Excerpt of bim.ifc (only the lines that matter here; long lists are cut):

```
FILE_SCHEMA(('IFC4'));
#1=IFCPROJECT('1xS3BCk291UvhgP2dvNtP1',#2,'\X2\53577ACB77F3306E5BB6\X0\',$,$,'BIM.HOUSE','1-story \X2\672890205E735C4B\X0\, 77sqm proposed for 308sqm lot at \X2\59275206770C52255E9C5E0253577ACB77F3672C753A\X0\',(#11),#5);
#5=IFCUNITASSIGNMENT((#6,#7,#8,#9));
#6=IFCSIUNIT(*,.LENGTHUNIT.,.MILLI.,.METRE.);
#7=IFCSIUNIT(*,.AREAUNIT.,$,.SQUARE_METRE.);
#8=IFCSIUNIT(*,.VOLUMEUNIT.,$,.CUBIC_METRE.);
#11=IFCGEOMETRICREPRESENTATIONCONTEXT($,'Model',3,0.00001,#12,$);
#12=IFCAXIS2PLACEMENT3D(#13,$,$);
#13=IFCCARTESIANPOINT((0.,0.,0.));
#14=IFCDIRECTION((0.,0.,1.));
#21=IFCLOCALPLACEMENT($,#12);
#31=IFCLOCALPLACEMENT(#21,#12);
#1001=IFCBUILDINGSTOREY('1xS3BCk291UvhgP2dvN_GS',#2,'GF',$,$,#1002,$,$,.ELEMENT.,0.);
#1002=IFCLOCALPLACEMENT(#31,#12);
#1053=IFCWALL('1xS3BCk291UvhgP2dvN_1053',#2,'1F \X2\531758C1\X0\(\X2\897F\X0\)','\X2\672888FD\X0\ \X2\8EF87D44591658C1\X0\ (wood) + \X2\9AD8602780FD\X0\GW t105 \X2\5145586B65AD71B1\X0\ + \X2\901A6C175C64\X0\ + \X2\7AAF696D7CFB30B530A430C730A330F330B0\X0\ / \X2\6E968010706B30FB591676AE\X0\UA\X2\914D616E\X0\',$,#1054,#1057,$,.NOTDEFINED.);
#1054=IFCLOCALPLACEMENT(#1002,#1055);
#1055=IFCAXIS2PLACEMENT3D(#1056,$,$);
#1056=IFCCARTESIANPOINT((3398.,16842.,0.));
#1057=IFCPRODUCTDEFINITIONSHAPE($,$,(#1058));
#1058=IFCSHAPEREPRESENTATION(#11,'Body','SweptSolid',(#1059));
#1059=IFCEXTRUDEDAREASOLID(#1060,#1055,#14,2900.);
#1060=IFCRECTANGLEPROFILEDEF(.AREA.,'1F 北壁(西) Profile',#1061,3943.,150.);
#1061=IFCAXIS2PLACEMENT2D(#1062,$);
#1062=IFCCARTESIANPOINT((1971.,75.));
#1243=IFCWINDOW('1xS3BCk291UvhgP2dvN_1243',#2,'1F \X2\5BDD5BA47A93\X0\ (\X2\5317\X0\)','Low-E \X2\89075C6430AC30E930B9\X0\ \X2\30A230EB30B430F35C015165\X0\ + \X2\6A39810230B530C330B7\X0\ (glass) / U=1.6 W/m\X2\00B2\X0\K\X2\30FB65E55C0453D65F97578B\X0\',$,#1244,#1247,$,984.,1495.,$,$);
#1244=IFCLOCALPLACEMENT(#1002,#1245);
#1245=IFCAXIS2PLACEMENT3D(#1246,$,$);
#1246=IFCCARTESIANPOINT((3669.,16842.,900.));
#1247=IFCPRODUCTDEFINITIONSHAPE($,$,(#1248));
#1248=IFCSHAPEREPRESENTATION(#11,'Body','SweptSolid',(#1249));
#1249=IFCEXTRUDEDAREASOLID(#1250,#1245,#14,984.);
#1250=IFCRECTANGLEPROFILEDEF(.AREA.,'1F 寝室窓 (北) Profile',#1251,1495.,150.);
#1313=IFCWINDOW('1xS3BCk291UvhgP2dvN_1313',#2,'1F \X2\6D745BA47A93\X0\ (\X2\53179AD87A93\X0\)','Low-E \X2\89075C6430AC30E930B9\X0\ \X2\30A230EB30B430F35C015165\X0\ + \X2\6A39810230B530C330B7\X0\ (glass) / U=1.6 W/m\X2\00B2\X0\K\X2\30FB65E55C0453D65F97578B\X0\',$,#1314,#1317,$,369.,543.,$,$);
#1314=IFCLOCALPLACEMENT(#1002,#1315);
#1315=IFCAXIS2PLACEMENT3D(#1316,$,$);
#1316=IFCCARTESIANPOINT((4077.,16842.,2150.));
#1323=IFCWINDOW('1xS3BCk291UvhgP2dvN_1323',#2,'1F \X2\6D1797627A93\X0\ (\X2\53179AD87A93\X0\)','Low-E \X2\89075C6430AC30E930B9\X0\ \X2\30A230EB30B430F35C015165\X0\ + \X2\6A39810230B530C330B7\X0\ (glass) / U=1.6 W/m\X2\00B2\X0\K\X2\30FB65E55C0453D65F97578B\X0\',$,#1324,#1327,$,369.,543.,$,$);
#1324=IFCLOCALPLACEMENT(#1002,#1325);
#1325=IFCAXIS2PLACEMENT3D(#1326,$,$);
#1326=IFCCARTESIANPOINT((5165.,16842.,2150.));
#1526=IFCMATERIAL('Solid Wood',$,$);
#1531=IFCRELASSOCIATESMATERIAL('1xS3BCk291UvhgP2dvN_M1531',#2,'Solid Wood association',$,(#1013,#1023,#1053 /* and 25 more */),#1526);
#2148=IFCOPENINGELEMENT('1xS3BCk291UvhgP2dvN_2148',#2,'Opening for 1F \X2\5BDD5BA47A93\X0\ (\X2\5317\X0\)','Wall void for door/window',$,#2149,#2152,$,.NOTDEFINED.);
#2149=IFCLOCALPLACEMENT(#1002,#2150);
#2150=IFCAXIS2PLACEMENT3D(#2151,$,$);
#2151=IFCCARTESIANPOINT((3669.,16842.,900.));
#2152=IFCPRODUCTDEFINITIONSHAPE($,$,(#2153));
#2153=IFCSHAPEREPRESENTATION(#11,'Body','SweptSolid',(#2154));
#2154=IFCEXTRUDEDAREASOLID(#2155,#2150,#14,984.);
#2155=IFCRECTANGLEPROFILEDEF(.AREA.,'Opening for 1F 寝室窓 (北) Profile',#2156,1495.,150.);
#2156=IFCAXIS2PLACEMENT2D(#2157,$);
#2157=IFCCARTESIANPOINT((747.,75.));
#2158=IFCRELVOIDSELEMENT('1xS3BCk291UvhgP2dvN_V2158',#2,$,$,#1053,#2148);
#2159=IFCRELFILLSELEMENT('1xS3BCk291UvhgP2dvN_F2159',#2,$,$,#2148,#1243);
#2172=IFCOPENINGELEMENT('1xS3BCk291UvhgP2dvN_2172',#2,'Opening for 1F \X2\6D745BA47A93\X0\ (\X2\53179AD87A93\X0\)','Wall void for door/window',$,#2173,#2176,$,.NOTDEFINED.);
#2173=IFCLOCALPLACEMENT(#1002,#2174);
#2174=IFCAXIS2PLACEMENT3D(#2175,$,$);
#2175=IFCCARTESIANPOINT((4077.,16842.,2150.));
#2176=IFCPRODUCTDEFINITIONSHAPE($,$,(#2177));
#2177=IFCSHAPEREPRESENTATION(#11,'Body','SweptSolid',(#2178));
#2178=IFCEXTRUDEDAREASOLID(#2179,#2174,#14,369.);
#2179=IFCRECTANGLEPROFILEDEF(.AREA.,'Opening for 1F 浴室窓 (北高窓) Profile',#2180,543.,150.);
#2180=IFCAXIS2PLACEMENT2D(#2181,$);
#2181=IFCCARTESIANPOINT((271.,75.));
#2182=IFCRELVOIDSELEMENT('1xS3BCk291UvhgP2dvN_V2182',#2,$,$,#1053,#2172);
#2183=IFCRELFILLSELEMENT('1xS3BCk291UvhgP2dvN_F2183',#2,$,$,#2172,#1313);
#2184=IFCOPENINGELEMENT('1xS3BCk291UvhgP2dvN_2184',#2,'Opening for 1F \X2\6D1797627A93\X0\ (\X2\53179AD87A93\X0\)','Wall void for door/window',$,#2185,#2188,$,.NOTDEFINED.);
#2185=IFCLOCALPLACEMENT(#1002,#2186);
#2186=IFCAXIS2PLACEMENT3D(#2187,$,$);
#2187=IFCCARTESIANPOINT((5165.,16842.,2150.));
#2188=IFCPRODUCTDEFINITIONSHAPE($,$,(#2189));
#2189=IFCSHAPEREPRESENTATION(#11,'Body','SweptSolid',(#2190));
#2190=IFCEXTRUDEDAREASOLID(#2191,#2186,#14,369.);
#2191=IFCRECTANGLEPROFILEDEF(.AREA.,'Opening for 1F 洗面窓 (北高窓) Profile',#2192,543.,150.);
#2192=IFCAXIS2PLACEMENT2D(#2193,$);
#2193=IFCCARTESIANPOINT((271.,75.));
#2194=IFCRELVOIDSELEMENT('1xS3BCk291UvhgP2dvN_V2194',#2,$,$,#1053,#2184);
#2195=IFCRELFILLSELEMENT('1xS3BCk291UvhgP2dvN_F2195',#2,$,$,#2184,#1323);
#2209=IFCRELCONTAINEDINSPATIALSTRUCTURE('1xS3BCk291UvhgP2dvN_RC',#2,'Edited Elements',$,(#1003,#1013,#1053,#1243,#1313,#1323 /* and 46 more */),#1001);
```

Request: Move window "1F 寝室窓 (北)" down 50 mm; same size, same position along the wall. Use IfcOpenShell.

```python
import numpy as np
import ifcopenshell
import ifcopenshell.api.geometry
import ifcopenshell.util.placement
import ifcopenshell.util.unit

model = ifcopenshell.open("bim.ifc")
unit_scale = ifcopenshell.util.unit.calculate_unit_scale(model)

window = model.by_guid("1xS3BCk291UvhgP2dvN_1243")
opening = window.FillsVoids[0].RelatingOpeningElement
dz = -50.0

shift = np.array([0.0, 0.0, dz])
# The window is not placed relative to its opening, so move both.
for product in (opening, window):
    matrix = ifcopenshell.util.placement.get_local_placement(product.ObjectPlacement)
    matrix[:3, 3] += shift
    ifcopenshell.api.geometry.edit_object_placement(model, product=product, matrix=matrix, is_si=False)

print(f"moved by {dz * unit_scale:+.3f} m")

model.write("bim_edited.ifc")
```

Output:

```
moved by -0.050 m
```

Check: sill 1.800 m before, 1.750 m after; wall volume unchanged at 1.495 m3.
